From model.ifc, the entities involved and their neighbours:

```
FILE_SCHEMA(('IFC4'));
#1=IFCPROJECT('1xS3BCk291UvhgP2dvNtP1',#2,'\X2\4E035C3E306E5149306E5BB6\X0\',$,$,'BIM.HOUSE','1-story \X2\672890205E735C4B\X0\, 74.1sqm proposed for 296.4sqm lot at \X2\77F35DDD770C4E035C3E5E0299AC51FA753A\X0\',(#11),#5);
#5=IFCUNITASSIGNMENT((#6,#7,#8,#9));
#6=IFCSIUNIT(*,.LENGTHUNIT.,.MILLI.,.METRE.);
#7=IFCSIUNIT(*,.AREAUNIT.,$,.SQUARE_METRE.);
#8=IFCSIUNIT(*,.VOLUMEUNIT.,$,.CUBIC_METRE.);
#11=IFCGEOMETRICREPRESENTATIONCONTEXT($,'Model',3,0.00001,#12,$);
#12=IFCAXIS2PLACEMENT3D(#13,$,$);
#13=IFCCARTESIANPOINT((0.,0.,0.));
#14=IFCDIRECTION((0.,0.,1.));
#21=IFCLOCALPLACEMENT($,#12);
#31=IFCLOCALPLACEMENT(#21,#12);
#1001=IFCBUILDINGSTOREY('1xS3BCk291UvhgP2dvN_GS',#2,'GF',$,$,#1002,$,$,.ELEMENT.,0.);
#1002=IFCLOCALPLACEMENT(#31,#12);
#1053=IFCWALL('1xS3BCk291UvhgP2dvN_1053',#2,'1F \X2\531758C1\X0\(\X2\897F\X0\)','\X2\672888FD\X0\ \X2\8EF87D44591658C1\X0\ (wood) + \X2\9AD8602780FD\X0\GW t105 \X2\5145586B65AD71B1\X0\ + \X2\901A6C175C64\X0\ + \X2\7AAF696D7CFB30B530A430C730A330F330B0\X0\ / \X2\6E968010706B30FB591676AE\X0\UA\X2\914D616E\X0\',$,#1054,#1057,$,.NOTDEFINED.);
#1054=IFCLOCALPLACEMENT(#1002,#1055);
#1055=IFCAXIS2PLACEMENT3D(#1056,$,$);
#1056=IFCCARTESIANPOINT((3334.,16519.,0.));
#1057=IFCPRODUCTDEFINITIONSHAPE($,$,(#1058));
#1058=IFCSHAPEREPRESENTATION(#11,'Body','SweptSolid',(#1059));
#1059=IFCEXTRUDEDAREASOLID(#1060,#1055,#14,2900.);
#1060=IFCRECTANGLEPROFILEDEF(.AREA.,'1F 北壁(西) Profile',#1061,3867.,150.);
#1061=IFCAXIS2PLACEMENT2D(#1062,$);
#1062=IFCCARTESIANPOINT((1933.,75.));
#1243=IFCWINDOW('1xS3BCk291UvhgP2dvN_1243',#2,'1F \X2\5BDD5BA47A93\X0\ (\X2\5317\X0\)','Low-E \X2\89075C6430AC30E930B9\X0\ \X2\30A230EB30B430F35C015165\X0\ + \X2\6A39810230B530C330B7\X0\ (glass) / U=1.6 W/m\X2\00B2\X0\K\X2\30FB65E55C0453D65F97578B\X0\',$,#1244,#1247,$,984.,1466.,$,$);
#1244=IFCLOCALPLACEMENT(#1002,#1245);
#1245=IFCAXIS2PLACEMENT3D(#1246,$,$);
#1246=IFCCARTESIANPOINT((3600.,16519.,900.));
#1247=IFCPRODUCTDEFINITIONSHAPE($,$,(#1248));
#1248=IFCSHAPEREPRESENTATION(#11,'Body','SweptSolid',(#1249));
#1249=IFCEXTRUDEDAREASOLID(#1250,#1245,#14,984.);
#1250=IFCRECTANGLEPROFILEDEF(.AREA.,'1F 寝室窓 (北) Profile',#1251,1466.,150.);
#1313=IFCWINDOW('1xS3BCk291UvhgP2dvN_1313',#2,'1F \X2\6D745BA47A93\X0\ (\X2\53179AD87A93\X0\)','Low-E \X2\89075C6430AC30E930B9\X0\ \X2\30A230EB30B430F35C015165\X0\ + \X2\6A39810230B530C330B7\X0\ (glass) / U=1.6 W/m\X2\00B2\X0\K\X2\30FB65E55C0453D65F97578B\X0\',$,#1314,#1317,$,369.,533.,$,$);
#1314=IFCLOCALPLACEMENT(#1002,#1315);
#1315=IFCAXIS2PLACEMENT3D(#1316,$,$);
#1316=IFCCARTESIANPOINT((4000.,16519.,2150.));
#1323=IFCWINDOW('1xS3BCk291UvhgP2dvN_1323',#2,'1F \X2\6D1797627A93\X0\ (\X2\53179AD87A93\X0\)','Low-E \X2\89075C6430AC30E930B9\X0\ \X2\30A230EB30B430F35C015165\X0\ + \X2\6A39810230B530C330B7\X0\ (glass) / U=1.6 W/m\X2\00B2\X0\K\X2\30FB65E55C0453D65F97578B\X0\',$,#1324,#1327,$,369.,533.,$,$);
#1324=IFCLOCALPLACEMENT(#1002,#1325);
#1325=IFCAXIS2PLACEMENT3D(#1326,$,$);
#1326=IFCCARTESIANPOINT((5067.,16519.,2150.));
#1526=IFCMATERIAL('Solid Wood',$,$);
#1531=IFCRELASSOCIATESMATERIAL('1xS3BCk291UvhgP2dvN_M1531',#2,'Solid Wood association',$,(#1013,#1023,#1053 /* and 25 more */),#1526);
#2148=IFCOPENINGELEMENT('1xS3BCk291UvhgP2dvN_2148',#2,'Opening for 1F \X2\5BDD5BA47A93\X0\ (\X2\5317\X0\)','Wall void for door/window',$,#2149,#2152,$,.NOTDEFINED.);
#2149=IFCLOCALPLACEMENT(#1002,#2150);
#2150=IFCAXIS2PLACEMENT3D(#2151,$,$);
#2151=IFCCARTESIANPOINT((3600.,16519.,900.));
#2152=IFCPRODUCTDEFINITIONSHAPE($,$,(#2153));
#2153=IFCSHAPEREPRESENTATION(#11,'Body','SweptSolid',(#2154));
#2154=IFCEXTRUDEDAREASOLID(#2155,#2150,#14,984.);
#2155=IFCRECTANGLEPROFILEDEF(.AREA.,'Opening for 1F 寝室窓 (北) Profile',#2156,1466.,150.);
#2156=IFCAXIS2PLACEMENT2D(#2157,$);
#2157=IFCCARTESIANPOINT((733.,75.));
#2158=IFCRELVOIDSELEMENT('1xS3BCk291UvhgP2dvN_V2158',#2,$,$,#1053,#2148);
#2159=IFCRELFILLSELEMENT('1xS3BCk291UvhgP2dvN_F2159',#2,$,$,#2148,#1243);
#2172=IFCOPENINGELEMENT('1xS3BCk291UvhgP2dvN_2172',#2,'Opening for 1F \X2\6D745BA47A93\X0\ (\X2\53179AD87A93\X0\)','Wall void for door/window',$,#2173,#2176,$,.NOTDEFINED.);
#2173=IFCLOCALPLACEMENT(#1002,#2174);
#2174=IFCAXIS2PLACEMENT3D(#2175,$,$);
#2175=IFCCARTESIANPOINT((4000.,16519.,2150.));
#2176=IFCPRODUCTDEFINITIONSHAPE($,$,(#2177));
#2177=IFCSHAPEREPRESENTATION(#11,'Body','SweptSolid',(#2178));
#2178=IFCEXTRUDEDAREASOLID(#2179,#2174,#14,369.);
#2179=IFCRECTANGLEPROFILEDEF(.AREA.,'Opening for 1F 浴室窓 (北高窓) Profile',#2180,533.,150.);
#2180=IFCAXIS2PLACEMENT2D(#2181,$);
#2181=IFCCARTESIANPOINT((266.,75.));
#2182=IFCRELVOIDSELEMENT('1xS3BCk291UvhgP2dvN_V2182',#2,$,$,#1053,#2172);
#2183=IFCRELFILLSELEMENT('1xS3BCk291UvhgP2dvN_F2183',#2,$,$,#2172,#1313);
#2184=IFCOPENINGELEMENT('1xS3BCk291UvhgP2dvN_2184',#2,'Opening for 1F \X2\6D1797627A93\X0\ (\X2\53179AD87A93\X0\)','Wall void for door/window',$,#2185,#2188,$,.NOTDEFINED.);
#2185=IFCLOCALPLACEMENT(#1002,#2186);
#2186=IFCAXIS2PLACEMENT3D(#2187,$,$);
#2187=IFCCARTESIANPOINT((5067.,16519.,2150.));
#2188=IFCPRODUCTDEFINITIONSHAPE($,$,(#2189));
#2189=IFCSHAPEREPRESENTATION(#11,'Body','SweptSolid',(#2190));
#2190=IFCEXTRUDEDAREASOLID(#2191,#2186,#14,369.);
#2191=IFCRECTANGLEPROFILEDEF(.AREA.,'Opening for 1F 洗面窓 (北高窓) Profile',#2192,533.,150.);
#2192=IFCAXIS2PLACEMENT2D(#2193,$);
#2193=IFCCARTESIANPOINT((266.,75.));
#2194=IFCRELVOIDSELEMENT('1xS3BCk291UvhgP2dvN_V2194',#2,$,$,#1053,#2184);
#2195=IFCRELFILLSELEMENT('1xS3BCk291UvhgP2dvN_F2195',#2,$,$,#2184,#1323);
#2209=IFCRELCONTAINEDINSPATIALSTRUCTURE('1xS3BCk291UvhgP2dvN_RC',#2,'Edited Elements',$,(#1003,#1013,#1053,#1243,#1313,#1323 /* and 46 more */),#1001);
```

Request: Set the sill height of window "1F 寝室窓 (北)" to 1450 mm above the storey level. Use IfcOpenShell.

```python
import numpy as np
import ifcopenshell
import ifcopenshell.api.geometry
import ifcopenshell.geom
import ifcopenshell.util.element
import ifcopenshell.util.placement
import ifcopenshell.util.shape
import ifcopenshell.util.unit

model = ifcopenshell.open("model.ifc")
unit_scale = ifcopenshell.util.unit.calculate_unit_scale(model)

window = model.by_id(1243)
opening = window.FillsVoids[0].RelatingOpeningElement
storey = ifcopenshell.util.element.get_container(window, ifc_class="IfcBuildingStorey")
level = ifcopenshell.util.placement.get_local_placement(storey.ObjectPlacement)[2, 3]

# The opening's origin need not be at the sill, so measure its lowest point.
shape = ifcopenshell.geom.create_shape(ifcopenshell.geom.settings(), opening)
bottom = ifcopenshell.util.shape.get_shape_bottom_elevation(shape, shape.geometry) / unit_scale
dz = level + 1.45 / unit_scale - bottom

shift = np.array([0.0, 0.0, dz])
# The window is not placed relative to its opening, so move both.
for product in (opening, window):
    matrix = ifcopenshell.util.placement.get_local_placement(product.ObjectPlacement)
    matrix[:3, 3] += shift
    ifcopenshell.api.geometry.edit_object_placement(model, product=product, matrix=matrix, is_si=False)

print(f"moved by {dz * unit_scale:+.3f} m")

model.write("model_edited.ifc")
```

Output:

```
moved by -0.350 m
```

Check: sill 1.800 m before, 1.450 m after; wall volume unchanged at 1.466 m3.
